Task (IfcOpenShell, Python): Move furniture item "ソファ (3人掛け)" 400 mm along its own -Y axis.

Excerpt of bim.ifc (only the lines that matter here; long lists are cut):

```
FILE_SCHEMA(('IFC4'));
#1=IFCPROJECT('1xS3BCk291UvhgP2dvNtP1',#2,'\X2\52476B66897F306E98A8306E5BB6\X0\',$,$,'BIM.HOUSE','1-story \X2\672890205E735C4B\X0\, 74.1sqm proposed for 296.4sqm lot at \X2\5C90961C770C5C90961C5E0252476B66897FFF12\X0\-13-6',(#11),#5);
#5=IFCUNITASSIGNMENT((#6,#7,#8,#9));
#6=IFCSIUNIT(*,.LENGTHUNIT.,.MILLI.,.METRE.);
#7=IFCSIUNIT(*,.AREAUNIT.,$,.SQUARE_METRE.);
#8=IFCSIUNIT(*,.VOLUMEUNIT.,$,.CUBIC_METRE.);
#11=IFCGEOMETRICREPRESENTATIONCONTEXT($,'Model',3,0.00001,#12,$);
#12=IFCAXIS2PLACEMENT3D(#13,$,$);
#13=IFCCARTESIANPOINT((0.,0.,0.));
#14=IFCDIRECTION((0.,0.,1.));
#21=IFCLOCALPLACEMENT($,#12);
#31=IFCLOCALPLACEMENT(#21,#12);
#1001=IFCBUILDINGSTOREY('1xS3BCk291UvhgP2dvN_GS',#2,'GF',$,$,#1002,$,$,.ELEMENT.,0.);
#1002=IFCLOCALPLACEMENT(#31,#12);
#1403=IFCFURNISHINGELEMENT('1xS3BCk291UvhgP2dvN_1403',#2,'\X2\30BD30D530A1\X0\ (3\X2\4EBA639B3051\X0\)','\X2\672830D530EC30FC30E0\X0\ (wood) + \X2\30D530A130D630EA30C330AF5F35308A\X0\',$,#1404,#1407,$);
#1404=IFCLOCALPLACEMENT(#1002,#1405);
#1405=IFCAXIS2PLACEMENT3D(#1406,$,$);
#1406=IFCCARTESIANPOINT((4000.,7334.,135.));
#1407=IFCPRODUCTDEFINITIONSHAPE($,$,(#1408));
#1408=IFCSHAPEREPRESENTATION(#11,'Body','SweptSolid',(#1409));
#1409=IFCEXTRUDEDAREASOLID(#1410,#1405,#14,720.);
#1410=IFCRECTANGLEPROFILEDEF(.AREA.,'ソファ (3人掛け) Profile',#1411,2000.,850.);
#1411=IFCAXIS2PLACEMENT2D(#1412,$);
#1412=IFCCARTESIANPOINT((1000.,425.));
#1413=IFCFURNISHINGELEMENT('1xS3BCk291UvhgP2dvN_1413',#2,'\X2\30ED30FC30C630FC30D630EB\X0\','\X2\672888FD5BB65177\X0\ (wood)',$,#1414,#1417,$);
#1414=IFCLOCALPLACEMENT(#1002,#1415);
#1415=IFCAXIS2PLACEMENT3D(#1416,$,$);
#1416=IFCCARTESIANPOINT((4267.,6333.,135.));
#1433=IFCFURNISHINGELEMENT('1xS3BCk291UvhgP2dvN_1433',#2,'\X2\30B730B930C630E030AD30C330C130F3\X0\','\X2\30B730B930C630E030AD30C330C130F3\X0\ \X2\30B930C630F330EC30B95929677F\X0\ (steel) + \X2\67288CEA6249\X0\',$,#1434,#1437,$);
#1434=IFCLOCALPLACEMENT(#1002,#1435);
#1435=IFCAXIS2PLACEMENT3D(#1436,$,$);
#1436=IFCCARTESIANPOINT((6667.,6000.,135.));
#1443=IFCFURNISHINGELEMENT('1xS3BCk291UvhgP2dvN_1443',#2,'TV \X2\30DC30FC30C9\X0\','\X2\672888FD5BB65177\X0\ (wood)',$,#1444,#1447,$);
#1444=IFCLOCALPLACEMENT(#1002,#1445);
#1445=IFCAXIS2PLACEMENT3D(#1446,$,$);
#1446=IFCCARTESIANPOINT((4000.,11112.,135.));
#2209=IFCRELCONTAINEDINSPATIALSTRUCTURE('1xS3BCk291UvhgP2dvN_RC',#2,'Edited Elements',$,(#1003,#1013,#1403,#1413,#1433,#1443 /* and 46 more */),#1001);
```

```python
import ifcopenshell
import ifcopenshell.api.geometry
import ifcopenshell.util.placement
import ifcopenshell.util.unit

model = ifcopenshell.open("bim.ifc")
unit_scale = ifcopenshell.util.unit.calculate_unit_scale(model)

item = model.by_guid("1xS3BCk291UvhgP2dvN_1403")
matrix = ifcopenshell.util.placement.get_local_placement(item.ObjectPlacement)
matrix[:3, 3] -= matrix[:3, 1] * 0.4 / unit_scale
ifcopenshell.api.geometry.edit_object_placement(model, product=item, matrix=matrix, is_si=False)

print(ifcopenshell.util.placement.get_local_placement(item.ObjectPlacement).round(3) + 0.0)

model.write("bim_rev.ifc")
```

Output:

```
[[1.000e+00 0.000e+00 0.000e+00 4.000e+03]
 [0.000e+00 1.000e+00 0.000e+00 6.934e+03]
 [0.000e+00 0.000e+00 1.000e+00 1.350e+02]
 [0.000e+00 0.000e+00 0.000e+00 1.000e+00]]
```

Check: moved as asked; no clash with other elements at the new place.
